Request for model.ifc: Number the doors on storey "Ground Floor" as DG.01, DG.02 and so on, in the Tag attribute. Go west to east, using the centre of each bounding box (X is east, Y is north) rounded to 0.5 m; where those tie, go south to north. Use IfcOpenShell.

First a look at what the model holds.

```python
import ifcopenshell
import ifcopenshell.util.element
import ifcopenshell.util.placement

model = ifcopenshell.open("model.ifc")
print(model.schema)
storey = next(s for s in model.by_type("IfcBuildingStorey") if s.Name == "Ground Floor")
doors = [e for e in ifcopenshell.util.element.get_decomposition(storey) if e.is_a("IfcDoor")]
for e in sorted(doors, key=lambda e: e.id()):
    origin = ifcopenshell.util.placement.get_local_placement(e.ObjectPlacement)[:3, 3]
    print(e.id(), e.Tag, e.Name, origin.round(2) + 0.0, sep=" | ")
```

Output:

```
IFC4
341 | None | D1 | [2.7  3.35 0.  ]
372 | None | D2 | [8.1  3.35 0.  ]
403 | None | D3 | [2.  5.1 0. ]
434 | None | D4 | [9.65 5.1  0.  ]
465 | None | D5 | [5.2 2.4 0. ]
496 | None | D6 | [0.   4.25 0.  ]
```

```python
import ifcopenshell
import ifcopenshell.geom
import ifcopenshell.util.element
import ifcopenshell.util.shape

model = ifcopenshell.open("model.ifc")
settings = ifcopenshell.geom.settings()
settings.set("use-world-coords", True)


def centre(element):
    shape = ifcopenshell.geom.create_shape(settings, element)
    return ifcopenshell.util.shape.get_bbox_centroid(shape.geometry)


storey = next(s for s in model.by_type("IfcBuildingStorey") if s.Name == "Ground Floor")
doors = [e for e in ifcopenshell.util.element.get_decomposition(storey) if e.is_a("IfcDoor")]

# Insertion points can sit at a corner or the storey origin, so sort by the geometry (in metres).
centres = {e: centre(e) for e in doors}
doors.sort(key=lambda e: (round(centres[e][0] / 0.5), centres[e][1]))

for i, e in enumerate(doors, start=1):
    number = f"DG.{i:02d}"
    e.Tag = number
    print(e.id(), number)

model.write("model_edited.ifc")
```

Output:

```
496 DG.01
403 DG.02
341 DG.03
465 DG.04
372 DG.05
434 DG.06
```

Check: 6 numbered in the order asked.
